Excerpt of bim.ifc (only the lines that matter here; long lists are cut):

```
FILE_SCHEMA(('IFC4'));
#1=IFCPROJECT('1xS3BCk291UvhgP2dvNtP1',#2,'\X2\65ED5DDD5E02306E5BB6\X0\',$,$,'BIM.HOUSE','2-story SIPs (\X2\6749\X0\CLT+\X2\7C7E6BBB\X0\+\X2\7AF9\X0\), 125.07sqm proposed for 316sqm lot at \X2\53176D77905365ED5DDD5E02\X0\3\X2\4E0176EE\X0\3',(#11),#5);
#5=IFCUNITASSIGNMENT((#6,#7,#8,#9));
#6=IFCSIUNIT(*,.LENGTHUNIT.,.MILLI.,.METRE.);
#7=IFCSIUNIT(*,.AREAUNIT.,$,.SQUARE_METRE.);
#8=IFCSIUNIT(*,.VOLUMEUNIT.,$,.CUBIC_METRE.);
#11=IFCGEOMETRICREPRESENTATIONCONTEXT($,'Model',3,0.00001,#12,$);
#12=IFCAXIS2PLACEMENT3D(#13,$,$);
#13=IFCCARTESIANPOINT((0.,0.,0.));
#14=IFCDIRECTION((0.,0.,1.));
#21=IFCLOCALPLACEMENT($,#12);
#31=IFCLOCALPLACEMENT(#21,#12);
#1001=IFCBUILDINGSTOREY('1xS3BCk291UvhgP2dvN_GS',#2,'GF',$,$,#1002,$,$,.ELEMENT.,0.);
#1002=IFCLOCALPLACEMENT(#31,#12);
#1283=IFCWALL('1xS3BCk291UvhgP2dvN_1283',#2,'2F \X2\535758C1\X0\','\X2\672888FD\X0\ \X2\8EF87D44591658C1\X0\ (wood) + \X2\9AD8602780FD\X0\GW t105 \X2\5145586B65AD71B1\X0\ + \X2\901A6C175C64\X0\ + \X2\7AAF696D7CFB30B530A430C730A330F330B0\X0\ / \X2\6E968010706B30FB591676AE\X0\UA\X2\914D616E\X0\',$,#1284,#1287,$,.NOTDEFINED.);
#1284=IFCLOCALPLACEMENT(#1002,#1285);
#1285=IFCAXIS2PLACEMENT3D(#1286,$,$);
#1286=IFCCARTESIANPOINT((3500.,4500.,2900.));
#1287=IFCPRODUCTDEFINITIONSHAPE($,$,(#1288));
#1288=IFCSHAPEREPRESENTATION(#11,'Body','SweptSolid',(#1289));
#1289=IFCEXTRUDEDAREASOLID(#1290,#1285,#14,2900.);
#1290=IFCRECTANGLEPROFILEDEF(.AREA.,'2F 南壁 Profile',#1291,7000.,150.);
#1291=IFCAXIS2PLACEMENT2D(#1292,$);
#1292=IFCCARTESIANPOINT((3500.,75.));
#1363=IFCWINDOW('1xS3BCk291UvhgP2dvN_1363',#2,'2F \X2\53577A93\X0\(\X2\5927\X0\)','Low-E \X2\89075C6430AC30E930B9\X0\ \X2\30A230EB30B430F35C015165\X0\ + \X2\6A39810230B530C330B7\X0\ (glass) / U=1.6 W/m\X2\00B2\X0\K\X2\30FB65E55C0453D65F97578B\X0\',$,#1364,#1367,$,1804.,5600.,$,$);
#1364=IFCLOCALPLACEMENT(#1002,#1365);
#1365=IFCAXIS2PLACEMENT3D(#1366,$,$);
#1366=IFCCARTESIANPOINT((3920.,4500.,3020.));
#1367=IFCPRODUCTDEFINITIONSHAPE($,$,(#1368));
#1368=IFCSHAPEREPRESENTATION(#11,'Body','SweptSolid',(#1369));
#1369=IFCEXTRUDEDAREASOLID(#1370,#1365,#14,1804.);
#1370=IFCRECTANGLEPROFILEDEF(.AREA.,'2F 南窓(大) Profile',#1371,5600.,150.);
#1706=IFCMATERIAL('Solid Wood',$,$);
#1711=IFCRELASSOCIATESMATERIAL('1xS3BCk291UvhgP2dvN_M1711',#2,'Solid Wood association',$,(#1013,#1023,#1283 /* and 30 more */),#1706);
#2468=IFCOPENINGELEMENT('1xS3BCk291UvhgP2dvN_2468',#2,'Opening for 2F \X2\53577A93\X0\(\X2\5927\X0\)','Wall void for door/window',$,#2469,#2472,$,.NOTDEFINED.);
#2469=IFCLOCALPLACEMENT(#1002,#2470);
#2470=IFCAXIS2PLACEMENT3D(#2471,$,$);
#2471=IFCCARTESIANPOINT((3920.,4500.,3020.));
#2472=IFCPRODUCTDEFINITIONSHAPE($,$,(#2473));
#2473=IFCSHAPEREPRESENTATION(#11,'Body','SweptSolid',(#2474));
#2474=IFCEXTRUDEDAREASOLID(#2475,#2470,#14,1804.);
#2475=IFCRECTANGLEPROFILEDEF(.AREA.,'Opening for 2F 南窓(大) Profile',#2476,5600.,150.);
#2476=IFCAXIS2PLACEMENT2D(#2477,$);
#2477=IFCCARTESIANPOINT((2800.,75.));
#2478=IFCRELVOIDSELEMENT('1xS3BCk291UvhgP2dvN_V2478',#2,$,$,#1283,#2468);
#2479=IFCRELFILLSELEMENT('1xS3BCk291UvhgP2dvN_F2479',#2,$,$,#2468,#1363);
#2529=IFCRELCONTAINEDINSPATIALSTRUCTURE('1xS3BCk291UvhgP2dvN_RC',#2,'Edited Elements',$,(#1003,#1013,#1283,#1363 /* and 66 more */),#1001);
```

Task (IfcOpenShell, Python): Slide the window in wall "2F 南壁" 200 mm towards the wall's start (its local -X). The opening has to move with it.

```python
import ifcopenshell
import ifcopenshell.api.geometry
import ifcopenshell.util.placement
import ifcopenshell.util.unit

model = ifcopenshell.open("bim.ifc")
unit_scale = ifcopenshell.util.unit.calculate_unit_scale(model)

window = model.by_id(1363)
opening = window.FillsVoids[0].RelatingOpeningElement
wall = opening.VoidsElements[0].RelatingBuildingElement

wall_matrix = ifcopenshell.util.placement.get_local_placement(wall.ObjectPlacement)
shift = wall_matrix[:3, 0] * -0.2 / unit_scale
before = ifcopenshell.util.placement.get_local_placement(window.ObjectPlacement)[:3, 3].copy()

# The window is not placed relative to its opening, so move both.
for product in (opening, window):
    matrix = ifcopenshell.util.placement.get_local_placement(product.ObjectPlacement)
    matrix[:3, 3] += shift
    ifcopenshell.api.geometry.edit_object_placement(model, product=product, matrix=matrix, is_si=False)

after = ifcopenshell.util.placement.get_local_placement(window.ObjectPlacement)[:3, 3]
print("window moved by", (after - before).round(3) + 0.0)

model.write("bim-out.ifc")
```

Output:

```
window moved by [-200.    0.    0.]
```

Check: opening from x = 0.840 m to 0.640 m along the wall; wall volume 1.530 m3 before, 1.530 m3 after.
